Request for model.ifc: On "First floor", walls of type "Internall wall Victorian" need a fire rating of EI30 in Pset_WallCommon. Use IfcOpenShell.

First a look at what the model holds.

```python
import ifcopenshell
import ifcopenshell.util.element

model = ifcopenshell.open("model.ifc")
print(model.schema)
storey = next(s for s in model.by_type("IfcBuildingStorey") if s.Name == "First floor")
walls = [e for e in ifcopenshell.util.element.get_decomposition(storey) if e.is_a("IfcWall")]
seen = {}
for e in walls:
    element_type = ifcopenshell.util.element.get_type(e)
    key = (element_type.Name if element_type != e and element_type else None, ifcopenshell.util.element.get_pset(e, "Pset_WallCommon", "FireRating"))
    seen[key] = seen.get(key, 0) + 1
for (name, value), count in sorted(seen.items(), key=str):
    print(count, "x", name, "|", value)
```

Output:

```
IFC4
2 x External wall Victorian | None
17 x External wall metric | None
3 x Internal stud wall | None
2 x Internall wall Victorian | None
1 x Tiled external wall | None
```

```python
import ifcopenshell
import ifcopenshell.api.pset
import ifcopenshell.util.element

model = ifcopenshell.open("model.ifc")

storey = next(s for s in model.by_type("IfcBuildingStorey") if s.Name == "First floor")
walls = [e for e in ifcopenshell.util.element.get_decomposition(storey) if e.is_a("IfcWall")]

count = 0
for e in walls:
    element_type = ifcopenshell.util.element.get_type(e)
    if element_type in (None, e) or element_type.Name != "Internall wall Victorian":
        continue
    # add_pset returns the element's existing set when there is one.
    pset = ifcopenshell.api.pset.add_pset(model, product=e, name="Pset_WallCommon")
    ifcopenshell.api.pset.edit_pset(model, pset=pset, properties={"FireRating": "EI30"})
    count += 1

print(count, "walls updated")

model.write("model-out.ifc")
```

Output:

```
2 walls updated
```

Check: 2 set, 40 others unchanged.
